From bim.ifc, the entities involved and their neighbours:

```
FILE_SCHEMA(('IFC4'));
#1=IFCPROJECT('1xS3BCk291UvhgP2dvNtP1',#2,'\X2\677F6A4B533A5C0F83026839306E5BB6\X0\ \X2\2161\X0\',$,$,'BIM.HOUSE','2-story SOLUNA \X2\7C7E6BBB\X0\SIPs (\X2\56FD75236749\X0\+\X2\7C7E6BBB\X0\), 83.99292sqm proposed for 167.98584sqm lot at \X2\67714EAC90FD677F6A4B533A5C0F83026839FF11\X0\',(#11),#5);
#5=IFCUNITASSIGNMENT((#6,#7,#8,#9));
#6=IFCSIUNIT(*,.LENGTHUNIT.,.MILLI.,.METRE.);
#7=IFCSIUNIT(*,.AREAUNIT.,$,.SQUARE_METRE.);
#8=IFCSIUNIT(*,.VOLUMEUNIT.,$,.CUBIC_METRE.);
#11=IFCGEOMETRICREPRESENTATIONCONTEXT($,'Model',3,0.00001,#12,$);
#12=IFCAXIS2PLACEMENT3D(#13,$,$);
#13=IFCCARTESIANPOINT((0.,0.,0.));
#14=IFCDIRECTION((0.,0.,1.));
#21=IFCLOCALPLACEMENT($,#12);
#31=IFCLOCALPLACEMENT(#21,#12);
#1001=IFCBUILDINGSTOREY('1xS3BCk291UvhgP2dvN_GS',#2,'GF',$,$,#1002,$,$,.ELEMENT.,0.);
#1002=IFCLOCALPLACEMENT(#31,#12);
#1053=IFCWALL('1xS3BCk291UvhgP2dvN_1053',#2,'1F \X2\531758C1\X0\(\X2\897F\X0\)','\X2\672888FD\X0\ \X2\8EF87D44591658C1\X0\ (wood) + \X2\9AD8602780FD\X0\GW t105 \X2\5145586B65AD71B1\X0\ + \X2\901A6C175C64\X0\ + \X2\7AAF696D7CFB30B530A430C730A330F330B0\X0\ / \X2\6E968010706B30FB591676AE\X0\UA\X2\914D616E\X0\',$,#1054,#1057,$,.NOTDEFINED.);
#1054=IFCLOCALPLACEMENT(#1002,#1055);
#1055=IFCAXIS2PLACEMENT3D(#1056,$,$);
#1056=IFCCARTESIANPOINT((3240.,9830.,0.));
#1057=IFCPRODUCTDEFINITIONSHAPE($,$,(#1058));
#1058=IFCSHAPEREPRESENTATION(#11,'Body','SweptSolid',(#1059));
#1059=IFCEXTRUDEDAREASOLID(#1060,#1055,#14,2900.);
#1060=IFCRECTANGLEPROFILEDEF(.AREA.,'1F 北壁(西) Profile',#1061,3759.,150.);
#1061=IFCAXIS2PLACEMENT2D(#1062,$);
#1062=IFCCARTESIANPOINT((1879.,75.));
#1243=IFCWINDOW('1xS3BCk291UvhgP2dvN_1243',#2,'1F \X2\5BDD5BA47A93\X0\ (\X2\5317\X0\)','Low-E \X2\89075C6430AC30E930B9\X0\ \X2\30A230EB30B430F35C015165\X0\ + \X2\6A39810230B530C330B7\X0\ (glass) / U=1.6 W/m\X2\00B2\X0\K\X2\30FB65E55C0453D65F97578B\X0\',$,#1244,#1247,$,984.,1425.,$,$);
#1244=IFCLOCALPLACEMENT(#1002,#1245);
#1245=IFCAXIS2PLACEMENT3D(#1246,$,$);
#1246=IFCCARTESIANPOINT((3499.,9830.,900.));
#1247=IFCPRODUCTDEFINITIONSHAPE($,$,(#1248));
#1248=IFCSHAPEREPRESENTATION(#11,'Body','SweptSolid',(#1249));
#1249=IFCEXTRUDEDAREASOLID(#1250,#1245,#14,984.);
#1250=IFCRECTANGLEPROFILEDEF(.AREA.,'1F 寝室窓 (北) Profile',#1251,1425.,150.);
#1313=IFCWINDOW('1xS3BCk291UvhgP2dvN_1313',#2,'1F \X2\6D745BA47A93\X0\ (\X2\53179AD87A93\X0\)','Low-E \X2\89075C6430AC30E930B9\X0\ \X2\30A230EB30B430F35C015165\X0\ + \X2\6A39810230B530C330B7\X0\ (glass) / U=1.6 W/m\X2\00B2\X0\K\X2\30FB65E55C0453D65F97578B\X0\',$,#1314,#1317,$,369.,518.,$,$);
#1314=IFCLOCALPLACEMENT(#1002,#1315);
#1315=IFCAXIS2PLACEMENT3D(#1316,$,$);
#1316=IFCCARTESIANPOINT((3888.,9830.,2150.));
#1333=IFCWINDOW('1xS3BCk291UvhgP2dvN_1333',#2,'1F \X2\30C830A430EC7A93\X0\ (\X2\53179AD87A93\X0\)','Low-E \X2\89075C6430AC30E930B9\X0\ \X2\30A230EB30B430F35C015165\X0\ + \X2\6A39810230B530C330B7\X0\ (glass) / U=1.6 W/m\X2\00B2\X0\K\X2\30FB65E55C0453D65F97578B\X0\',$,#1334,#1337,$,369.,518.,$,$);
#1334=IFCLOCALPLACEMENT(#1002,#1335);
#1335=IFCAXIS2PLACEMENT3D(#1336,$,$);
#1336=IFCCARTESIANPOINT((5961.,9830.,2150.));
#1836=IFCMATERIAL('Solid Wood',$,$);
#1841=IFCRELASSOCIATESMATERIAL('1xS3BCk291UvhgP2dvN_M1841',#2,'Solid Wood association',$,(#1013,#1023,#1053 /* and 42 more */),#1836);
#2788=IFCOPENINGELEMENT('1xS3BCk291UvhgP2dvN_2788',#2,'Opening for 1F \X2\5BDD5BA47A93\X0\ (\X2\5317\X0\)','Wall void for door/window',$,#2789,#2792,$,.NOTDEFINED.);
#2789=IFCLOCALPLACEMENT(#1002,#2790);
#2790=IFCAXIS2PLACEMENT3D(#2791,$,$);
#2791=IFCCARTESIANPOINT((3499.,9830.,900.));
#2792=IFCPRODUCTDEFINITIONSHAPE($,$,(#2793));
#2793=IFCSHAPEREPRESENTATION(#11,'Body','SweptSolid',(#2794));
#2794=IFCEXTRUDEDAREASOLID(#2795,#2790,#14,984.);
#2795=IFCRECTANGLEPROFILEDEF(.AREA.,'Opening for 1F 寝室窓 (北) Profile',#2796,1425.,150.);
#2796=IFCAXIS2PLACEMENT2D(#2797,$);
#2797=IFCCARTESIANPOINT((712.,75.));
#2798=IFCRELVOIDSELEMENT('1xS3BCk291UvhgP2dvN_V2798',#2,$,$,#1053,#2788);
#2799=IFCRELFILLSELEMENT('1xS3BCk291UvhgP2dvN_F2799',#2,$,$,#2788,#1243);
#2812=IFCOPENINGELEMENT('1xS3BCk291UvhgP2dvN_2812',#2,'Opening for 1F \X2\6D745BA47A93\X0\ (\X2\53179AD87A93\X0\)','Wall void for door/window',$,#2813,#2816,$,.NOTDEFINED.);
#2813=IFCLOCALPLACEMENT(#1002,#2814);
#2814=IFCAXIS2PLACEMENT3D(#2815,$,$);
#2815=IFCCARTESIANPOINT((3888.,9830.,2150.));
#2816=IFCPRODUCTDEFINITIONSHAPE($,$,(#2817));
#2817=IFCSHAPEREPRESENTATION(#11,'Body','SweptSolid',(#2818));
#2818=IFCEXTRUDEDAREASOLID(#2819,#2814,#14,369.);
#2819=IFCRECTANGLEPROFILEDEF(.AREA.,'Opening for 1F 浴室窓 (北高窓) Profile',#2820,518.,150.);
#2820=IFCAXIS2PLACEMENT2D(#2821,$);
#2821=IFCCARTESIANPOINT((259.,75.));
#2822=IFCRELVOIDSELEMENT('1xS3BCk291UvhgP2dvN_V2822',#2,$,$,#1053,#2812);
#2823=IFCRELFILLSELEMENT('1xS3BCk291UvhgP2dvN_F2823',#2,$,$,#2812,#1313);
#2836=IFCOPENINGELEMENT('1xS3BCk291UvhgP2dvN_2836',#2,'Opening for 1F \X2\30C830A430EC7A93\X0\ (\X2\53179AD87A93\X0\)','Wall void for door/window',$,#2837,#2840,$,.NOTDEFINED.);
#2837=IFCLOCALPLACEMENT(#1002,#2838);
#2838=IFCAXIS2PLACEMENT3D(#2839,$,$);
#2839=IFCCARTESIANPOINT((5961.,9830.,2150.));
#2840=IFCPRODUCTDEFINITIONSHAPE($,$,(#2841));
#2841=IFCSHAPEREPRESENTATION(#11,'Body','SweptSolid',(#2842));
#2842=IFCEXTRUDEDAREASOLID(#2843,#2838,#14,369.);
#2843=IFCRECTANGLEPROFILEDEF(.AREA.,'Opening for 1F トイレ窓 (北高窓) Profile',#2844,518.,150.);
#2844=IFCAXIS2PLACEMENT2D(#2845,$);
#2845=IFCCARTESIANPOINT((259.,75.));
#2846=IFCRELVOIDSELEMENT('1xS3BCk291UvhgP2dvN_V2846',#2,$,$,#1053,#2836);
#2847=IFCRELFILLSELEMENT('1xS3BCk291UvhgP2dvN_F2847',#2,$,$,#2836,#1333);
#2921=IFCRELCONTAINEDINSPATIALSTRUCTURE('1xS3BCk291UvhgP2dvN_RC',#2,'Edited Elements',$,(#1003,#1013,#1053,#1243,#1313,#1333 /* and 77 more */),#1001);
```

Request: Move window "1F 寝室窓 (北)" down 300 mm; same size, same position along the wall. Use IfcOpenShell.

```python
import numpy as np
import ifcopenshell
import ifcopenshell.api.geometry
import ifcopenshell.util.placement
import ifcopenshell.util.unit

model = ifcopenshell.open("bim.ifc")
unit_scale = ifcopenshell.util.unit.calculate_unit_scale(model)

window = model.by_id(1243)
opening = window.FillsVoids[0].RelatingOpeningElement
dz = -300.0

shift = np.array([0.0, 0.0, dz])
# The window is not placed relative to its opening, so move both.
for product in (opening, window):
    matrix = ifcopenshell.util.placement.get_local_placement(product.ObjectPlacement)
    matrix[:3, 3] += shift
    ifcopenshell.api.geometry.edit_object_placement(model, product=product, matrix=matrix, is_si=False)

print(f"moved by {dz * unit_scale:+.3f} m")

model.write("bim_updated.ifc")
```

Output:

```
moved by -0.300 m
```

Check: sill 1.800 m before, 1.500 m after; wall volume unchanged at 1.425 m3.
